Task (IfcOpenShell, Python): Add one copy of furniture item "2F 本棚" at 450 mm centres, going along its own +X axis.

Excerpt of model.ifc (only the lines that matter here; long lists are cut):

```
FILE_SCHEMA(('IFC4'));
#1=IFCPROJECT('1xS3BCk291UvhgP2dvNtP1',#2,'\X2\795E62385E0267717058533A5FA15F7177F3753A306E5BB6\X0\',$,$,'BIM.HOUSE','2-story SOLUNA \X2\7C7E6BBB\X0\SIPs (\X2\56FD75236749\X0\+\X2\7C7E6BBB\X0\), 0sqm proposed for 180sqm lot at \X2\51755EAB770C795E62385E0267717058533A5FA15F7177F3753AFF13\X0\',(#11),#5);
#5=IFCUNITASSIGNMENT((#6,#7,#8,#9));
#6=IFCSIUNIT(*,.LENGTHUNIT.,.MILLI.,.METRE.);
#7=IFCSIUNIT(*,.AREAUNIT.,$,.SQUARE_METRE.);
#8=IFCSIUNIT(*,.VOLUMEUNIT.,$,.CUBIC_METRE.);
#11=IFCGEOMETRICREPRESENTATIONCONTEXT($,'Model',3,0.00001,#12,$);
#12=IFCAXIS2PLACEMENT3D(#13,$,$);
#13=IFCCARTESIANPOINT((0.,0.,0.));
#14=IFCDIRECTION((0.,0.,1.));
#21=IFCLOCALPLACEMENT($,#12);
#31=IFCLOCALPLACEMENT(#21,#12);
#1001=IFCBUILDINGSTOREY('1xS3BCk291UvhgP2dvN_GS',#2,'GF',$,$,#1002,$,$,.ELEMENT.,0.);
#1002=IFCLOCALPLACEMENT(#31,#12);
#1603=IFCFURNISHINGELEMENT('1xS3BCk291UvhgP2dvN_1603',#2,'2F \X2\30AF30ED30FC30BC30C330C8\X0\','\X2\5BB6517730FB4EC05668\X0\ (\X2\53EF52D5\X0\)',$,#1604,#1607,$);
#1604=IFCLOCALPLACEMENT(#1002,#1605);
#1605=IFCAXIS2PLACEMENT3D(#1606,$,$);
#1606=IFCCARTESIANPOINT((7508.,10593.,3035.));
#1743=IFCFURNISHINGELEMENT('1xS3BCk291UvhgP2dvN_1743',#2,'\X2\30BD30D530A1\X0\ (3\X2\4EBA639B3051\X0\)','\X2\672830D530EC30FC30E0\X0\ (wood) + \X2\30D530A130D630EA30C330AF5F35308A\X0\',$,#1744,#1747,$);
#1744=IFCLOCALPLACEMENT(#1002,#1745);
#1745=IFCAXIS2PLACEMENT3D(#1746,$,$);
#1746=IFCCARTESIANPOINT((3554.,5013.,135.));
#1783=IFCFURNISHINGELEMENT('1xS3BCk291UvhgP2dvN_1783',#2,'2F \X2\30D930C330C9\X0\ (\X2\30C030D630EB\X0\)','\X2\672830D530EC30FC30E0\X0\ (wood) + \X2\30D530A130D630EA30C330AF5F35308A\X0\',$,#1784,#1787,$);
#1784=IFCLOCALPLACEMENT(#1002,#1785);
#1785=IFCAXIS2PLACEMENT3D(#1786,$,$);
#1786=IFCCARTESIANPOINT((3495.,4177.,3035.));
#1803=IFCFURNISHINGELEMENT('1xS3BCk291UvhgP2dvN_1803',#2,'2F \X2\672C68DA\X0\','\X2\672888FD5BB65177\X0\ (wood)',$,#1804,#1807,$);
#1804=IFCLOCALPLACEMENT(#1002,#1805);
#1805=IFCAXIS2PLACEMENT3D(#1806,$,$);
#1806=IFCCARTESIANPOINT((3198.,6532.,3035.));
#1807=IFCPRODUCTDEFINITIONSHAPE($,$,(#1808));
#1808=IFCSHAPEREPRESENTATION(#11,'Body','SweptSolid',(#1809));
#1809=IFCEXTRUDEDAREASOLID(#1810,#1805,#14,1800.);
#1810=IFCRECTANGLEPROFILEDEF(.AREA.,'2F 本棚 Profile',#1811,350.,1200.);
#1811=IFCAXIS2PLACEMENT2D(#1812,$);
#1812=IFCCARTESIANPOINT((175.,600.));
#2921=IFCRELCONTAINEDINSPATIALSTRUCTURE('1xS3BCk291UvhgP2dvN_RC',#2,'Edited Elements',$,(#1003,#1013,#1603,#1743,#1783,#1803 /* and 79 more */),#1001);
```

```python
import ifcopenshell
import ifcopenshell.api.geometry
import ifcopenshell.api.root
import ifcopenshell.util.element
import ifcopenshell.util.placement
import ifcopenshell.util.unit

model = ifcopenshell.open("model.ifc")
unit_scale = ifcopenshell.util.unit.calculate_unit_scale(model)


def reuse_history(source, copy):
    """copy_class also copies each property set's owner history, people and application; keep the originals."""
    for rel in copy.IsDefinedBy:
        if rel.is_a("IfcRelDefinesByProperties") and (history := rel.RelatingPropertyDefinition.OwnerHistory):
            rel.RelatingPropertyDefinition.OwnerHistory = source.OwnerHistory
            ifcopenshell.util.element.remove_deep2(model, history)


source = model.by_guid("1xS3BCk291UvhgP2dvN_1803")
base = ifcopenshell.util.placement.get_local_placement(source.ObjectPlacement)
step = base[:3, 0] * 0.45 / unit_scale

for i in range(1, 2):
    copy = ifcopenshell.api.root.copy_class(model, product=source)
    copy.Representation = ifcopenshell.util.element.copy_deep(
        model, source.Representation, exclude=["IfcGeometricRepresentationContext", "IfcRepresentationMap"]
    )
    reuse_history(source, copy)
    matrix = base.copy()
    matrix[:3, 3] += i * step
    print("added at", matrix[:3, 3].round(3) + 0.0)
    ifcopenshell.api.geometry.edit_object_placement(model, product=copy, matrix=matrix, is_si=False)

model.write("model_updated.ifc")
```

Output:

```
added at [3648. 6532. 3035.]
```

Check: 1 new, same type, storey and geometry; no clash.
